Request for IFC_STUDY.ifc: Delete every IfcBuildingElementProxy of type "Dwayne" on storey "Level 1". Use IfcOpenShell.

First a look at what the model holds.

```python
import ifcopenshell
import ifcopenshell.util.element

model = ifcopenshell.open("IFC_STUDY.ifc")
print(model.schema)
storey = next(s for s in model.by_type("IfcBuildingStorey") if s.Name == "Level 1")
proxies = [e for e in ifcopenshell.util.element.get_decomposition(storey) if e.is_a("IfcBuildingElementProxy")]
seen = {}
for e in proxies:
    element_type = ifcopenshell.util.element.get_type(e)
    name = element_type.Name if element_type not in (None, e) else None
    seen[name] = seen.get(name, 0) + 1
for name, count in sorted(seen.items(), key=str):
    print(count, "x", name)
```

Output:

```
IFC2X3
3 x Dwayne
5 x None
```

```python
import ifcopenshell
import ifcopenshell.api.root
import ifcopenshell.util.element

model = ifcopenshell.open("IFC_STUDY.ifc")

storey = next(s for s in model.by_type("IfcBuildingStorey") if s.Name == "Level 1")
proxies = [e for e in ifcopenshell.util.element.get_decomposition(storey) if e.is_a("IfcBuildingElementProxy")]
targets = [e for e in proxies if (t := ifcopenshell.util.element.get_type(e)) not in (None, e) and t.Name == "Dwayne"]

for e in targets:
    ifcopenshell.api.root.remove_product(model, product=e)
print(len(targets), "removed")

model.write("IFC_STUDY_edited.ifc")
```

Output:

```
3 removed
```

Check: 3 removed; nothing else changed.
